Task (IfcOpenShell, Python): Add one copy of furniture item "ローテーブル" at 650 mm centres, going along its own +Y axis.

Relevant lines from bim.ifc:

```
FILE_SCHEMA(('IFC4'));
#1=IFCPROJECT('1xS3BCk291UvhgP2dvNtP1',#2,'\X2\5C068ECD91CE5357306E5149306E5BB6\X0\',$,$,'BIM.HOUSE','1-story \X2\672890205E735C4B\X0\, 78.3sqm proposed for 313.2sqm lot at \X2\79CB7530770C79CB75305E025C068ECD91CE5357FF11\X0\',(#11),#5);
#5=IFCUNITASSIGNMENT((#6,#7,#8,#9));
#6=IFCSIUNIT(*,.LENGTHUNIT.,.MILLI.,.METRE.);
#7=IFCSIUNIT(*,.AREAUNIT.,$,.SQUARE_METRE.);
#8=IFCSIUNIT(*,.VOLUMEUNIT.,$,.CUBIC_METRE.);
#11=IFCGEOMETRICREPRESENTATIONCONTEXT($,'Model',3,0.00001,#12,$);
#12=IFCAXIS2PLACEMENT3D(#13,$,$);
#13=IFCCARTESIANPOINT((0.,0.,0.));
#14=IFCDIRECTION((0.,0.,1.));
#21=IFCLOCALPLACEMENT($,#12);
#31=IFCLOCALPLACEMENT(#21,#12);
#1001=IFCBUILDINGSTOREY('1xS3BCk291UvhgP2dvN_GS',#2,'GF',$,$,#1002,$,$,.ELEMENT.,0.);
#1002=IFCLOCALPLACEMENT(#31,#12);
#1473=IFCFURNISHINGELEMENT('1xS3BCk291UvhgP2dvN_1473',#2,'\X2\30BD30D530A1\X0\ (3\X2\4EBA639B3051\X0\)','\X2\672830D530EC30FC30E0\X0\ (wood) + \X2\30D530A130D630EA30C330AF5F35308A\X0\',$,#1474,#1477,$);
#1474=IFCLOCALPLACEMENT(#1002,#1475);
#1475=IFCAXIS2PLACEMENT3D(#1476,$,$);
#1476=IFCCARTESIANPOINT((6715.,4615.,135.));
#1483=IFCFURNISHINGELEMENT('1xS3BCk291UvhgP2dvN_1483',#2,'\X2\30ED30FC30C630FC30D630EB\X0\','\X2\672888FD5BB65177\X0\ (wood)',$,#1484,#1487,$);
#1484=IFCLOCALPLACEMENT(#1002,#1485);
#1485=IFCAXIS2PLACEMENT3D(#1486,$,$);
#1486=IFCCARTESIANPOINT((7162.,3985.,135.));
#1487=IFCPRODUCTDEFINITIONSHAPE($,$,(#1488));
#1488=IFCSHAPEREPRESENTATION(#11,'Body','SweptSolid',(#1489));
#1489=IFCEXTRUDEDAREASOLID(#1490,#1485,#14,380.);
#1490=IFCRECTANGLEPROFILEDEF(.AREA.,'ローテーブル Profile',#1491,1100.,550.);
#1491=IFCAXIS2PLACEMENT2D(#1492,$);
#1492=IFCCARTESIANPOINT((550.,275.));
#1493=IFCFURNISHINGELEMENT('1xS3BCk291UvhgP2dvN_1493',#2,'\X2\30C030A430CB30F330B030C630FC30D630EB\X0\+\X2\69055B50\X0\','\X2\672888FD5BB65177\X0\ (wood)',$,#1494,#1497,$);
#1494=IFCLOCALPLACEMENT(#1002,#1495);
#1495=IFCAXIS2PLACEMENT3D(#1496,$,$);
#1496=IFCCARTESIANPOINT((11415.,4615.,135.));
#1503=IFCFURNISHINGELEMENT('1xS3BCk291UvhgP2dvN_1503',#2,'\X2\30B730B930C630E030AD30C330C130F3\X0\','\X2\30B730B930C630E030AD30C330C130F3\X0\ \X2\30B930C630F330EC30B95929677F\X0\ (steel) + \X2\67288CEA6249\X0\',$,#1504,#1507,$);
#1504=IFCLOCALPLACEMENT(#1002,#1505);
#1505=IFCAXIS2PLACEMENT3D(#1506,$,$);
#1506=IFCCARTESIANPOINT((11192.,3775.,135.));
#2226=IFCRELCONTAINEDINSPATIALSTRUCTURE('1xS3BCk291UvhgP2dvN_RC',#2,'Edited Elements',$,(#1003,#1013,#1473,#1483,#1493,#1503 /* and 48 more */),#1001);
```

```python
import ifcopenshell
import ifcopenshell.api.geometry
import ifcopenshell.api.root
import ifcopenshell.util.element
import ifcopenshell.util.placement
import ifcopenshell.util.unit

model = ifcopenshell.open("bim.ifc")
unit_scale = ifcopenshell.util.unit.calculate_unit_scale(model)


def reuse_history(source, copy):
    """copy_class also copies each property set's owner history, people and application; keep the originals."""
    for rel in copy.IsDefinedBy:
        if rel.is_a("IfcRelDefinesByProperties") and (history := rel.RelatingPropertyDefinition.OwnerHistory):
            rel.RelatingPropertyDefinition.OwnerHistory = source.OwnerHistory
            ifcopenshell.util.element.remove_deep2(model, history)


source = model.by_guid("1xS3BCk291UvhgP2dvN_1483")
base = ifcopenshell.util.placement.get_local_placement(source.ObjectPlacement)
step = base[:3, 1] * 0.65 / unit_scale

for i in range(1, 2):
    copy = ifcopenshell.api.root.copy_class(model, product=source)
    copy.Representation = ifcopenshell.util.element.copy_deep(
        model, source.Representation, exclude=["IfcGeometricRepresentationContext", "IfcRepresentationMap"]
    )
    reuse_history(source, copy)
    matrix = base.copy()
    matrix[:3, 3] += i * step
    print("added at", matrix[:3, 3].round(3) + 0.0)
    ifcopenshell.api.geometry.edit_object_placement(model, product=copy, matrix=matrix, is_si=False)

model.write("bim_edited.ifc")
```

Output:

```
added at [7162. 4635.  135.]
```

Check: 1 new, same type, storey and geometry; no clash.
